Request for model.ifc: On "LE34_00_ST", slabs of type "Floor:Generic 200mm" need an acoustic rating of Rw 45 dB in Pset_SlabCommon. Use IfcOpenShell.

First a look at what the model holds.

```python
import ifcopenshell
import ifcopenshell.util.element

model = ifcopenshell.open("model.ifc")
print(model.schema)
storey = next(s for s in model.by_type("IfcBuildingStorey") if s.Name == "LE34_00_ST")
slabs = [e for e in ifcopenshell.util.element.get_decomposition(storey) if e.is_a("IfcSlab")]
seen = {}
for e in slabs:
    element_type = ifcopenshell.util.element.get_type(e)
    key = (element_type.Name if element_type != e and element_type else None, ifcopenshell.util.element.get_pset(e, "Pset_SlabCommon", "AcousticRating"))
    seen[key] = seen.get(key, 0) + 1
for (name, value), count in sorted(seen.items(), key=str):
    print(count, "x", name, "|", value)
```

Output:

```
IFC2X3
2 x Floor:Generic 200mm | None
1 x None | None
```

```python
import ifcopenshell
import ifcopenshell.api.pset
import ifcopenshell.util.element

model = ifcopenshell.open("model.ifc")

storey = next(s for s in model.by_type("IfcBuildingStorey") if s.Name == "LE34_00_ST")
slabs = [e for e in ifcopenshell.util.element.get_decomposition(storey) if e.is_a("IfcSlab")]

count = 0
for e in slabs:
    element_type = ifcopenshell.util.element.get_type(e)
    if element_type in (None, e) or element_type.Name != "Floor:Generic 200mm":
        continue
    # add_pset returns the element's existing set when there is one.
    pset = ifcopenshell.api.pset.add_pset(model, product=e, name="Pset_SlabCommon")
    ifcopenshell.api.pset.edit_pset(model, pset=pset, properties={"AcousticRating": "Rw 45 dB"})
    count += 1

print(count, "slabs updated")

model.write("model_v2.ifc")
```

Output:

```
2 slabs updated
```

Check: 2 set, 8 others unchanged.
